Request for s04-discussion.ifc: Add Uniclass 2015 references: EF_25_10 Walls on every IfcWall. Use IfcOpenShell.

First a look at what the model holds.

```python
import ifcopenshell

model = ifcopenshell.open("s04-discussion.ifc")
print(model.schema)
print("classifications:", [c.Name for c in model.by_type("IfcClassification")])
for ifc_class in ("IfcDoor", "IfcRoof", "IfcStair", "IfcWall", "IfcWindow"):
    print(ifc_class, len(model.by_type(ifc_class)))
```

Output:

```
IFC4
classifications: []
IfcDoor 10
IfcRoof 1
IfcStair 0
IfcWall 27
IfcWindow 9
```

```python
import ifcopenshell
import ifcopenshell.api.classification

model = ifcopenshell.open("s04-discussion.ifc")

system = ifcopenshell.api.classification.add_classification(model, classification="Uniclass 2015")

codes = {
    "IfcWall": ("EF_25_10", "Walls"),
}
for ifc_class, (code, name) in codes.items():
    products = model.by_type(ifc_class)
    ifcopenshell.api.classification.add_reference(
        model, products=products, classification=system, identification=code, name=name
    )
    print(code, len(products))

model.write("s04-discussion_rev.ifc")
```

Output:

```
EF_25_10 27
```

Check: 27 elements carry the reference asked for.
